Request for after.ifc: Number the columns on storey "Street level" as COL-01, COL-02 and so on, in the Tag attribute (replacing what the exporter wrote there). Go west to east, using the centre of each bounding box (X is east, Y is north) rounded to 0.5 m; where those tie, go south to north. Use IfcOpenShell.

First a look at what the model holds.

```python
import ifcopenshell
import ifcopenshell.util.element
import ifcopenshell.util.placement

model = ifcopenshell.open("after.ifc")
print(model.schema)
storey = next(s for s in model.by_type("IfcBuildingStorey") if s.Name == "Street level")
columns = [e for e in ifcopenshell.util.element.get_decomposition(storey) if e.is_a("IfcColumn")]
for e in sorted(columns, key=lambda e: e.id()):
    origin = ifcopenshell.util.placement.get_local_placement(e.ObjectPlacement)[:3, 3]
    print(e.id(), e.Tag, e.Name, origin.round(2) + 0.0, sep=" | ")
```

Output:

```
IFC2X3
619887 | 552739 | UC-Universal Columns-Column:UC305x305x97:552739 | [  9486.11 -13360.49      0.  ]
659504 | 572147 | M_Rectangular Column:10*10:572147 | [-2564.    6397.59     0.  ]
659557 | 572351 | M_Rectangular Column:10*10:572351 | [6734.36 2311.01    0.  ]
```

```python
import ifcopenshell
import ifcopenshell.geom
import ifcopenshell.util.element
import ifcopenshell.util.shape

model = ifcopenshell.open("after.ifc")
settings = ifcopenshell.geom.settings()
settings.set("use-world-coords", True)


def centre(element):
    shape = ifcopenshell.geom.create_shape(settings, element)
    return ifcopenshell.util.shape.get_bbox_centroid(shape.geometry)


storey = next(s for s in model.by_type("IfcBuildingStorey") if s.Name == "Street level")
columns = [e for e in ifcopenshell.util.element.get_decomposition(storey) if e.is_a("IfcColumn")]

# Insertion points can sit at a corner or the storey origin, so sort by the geometry (in metres).
centres = {e: centre(e) for e in columns}
columns.sort(key=lambda e: (round(centres[e][0] / 0.5), centres[e][1]))

for i, e in enumerate(columns, start=1):
    number = f"COL-{i:02d}"
    e.Tag = number
    print(e.id(), number)

model.write("after-out.ifc")
```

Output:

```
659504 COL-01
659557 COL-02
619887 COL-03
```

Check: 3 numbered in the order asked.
